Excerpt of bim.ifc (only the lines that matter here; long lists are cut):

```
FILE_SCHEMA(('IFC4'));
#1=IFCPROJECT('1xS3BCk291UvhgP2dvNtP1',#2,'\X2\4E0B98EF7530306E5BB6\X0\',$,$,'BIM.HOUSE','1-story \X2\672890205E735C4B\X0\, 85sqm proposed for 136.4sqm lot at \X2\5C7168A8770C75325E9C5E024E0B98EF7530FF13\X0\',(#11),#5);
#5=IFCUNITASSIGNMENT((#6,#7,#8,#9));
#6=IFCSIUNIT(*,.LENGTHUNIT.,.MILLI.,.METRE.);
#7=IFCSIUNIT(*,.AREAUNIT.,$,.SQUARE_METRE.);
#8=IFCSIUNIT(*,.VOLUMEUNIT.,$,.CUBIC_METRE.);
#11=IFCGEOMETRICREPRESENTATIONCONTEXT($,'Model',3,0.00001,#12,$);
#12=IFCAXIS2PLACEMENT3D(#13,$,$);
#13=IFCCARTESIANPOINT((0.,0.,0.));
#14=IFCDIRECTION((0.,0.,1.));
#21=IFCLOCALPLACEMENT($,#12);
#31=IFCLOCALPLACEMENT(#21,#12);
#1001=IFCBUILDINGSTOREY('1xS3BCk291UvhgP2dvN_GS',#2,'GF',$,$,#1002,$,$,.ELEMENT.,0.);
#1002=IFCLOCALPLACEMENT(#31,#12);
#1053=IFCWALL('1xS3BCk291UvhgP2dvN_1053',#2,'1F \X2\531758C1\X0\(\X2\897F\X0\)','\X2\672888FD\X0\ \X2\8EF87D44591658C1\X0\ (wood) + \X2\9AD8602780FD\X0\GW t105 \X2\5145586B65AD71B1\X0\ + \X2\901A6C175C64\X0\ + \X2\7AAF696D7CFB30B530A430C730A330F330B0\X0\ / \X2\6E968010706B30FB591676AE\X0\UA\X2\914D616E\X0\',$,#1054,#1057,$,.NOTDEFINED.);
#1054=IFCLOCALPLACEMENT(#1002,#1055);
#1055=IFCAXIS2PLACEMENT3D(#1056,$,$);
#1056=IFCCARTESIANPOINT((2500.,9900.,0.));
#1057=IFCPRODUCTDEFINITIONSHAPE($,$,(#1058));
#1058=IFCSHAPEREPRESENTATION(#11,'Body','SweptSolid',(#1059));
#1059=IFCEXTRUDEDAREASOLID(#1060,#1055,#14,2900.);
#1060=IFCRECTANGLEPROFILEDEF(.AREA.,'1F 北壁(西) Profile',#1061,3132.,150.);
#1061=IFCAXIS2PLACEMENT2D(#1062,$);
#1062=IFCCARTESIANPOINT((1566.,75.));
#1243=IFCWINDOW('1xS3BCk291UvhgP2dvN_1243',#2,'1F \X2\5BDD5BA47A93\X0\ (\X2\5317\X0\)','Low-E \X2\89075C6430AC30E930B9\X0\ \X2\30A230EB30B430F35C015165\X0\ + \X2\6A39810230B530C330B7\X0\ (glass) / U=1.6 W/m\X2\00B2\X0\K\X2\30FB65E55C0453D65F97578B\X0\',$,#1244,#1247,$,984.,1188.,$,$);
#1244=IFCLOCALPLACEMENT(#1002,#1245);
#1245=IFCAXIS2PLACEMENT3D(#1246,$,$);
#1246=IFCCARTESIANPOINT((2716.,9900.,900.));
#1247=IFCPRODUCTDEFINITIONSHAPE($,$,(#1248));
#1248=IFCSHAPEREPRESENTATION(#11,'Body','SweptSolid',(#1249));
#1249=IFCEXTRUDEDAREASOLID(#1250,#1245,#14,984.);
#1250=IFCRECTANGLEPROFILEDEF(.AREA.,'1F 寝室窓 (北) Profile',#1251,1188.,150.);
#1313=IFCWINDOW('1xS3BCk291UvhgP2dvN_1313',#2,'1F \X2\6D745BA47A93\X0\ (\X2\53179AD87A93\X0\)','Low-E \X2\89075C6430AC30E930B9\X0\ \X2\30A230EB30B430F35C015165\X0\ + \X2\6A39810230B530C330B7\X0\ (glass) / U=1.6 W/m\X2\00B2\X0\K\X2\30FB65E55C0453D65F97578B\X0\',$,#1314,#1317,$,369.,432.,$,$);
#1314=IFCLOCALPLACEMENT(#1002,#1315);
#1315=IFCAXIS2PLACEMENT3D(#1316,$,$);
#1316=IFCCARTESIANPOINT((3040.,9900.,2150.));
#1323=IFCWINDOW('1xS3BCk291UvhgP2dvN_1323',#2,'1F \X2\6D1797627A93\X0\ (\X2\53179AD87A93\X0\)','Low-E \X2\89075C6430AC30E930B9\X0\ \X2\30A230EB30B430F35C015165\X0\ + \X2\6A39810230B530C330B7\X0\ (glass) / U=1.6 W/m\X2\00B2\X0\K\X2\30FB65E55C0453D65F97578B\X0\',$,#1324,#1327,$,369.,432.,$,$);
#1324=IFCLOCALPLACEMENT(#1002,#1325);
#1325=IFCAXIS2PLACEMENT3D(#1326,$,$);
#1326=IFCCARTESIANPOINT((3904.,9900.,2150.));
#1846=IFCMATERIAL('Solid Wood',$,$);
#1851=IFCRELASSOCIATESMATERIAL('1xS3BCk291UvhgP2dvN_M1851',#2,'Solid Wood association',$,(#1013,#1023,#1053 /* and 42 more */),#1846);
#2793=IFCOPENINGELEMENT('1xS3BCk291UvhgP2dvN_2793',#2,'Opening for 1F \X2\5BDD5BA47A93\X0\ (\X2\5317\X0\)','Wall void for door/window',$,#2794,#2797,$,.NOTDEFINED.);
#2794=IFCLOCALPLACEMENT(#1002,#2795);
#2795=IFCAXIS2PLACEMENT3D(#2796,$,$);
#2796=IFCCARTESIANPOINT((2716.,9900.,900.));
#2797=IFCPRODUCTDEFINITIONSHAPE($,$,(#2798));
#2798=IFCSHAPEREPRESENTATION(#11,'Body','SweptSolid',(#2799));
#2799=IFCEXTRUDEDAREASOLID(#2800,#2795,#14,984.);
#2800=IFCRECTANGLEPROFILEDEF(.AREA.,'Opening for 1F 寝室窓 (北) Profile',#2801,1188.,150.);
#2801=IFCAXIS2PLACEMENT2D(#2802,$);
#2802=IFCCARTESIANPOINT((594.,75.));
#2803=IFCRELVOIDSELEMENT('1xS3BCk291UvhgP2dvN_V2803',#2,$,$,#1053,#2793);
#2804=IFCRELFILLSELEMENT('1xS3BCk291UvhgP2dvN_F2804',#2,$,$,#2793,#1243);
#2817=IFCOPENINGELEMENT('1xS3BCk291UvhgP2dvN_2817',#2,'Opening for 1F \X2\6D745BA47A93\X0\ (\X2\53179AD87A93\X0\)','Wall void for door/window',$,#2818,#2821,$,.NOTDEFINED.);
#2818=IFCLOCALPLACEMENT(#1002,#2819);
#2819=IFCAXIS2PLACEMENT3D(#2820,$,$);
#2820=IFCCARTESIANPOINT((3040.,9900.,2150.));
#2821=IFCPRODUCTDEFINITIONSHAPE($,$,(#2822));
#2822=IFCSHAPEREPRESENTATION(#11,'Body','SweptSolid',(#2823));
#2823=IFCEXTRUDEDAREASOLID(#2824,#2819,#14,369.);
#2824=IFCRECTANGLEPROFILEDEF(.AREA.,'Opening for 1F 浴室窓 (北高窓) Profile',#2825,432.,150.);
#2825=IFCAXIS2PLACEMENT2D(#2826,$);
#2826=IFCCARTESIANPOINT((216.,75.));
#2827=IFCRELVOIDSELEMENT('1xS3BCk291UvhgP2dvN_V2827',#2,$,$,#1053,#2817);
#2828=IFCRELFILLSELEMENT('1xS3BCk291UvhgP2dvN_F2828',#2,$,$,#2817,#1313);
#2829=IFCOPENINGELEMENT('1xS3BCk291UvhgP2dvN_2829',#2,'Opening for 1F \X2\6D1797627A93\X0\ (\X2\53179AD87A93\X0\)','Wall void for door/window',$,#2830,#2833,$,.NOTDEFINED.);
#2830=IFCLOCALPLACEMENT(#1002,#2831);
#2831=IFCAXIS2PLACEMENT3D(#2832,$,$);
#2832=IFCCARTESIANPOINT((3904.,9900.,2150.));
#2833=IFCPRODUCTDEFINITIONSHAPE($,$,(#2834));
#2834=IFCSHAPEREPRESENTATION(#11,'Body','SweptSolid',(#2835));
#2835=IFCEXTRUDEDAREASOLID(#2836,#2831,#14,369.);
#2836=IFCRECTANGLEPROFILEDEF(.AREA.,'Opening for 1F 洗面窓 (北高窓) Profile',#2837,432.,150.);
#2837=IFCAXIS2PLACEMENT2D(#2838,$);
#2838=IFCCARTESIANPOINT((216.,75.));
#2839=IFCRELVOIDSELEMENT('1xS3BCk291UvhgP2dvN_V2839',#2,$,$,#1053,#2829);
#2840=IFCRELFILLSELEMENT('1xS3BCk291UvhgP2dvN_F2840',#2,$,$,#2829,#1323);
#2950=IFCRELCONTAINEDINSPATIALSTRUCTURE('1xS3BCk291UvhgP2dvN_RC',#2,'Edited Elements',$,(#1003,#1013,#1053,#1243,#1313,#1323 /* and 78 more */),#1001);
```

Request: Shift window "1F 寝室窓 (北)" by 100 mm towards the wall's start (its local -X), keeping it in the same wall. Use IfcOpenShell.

```python
import ifcopenshell
import ifcopenshell.api.geometry
import ifcopenshell.util.placement
import ifcopenshell.util.unit

model = ifcopenshell.open("bim.ifc")
unit_scale = ifcopenshell.util.unit.calculate_unit_scale(model)

window = model.by_guid("1xS3BCk291UvhgP2dvN_1243")
opening = window.FillsVoids[0].RelatingOpeningElement
wall = opening.VoidsElements[0].RelatingBuildingElement

wall_matrix = ifcopenshell.util.placement.get_local_placement(wall.ObjectPlacement)
shift = wall_matrix[:3, 0] * -0.1 / unit_scale
before = ifcopenshell.util.placement.get_local_placement(window.ObjectPlacement)[:3, 3].copy()

# The window is not placed relative to its opening, so move both.
for product in (opening, window):
    matrix = ifcopenshell.util.placement.get_local_placement(product.ObjectPlacement)
    matrix[:3, 3] += shift
    ifcopenshell.api.geometry.edit_object_placement(model, product=product, matrix=matrix, is_si=False)

after = ifcopenshell.util.placement.get_local_placement(window.ObjectPlacement)[:3, 3]
print("window moved by", (after - before).round(3) + 0.0)

model.write("bim_updated.ifc")
```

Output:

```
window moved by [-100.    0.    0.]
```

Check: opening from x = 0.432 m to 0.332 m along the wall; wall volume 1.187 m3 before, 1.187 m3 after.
